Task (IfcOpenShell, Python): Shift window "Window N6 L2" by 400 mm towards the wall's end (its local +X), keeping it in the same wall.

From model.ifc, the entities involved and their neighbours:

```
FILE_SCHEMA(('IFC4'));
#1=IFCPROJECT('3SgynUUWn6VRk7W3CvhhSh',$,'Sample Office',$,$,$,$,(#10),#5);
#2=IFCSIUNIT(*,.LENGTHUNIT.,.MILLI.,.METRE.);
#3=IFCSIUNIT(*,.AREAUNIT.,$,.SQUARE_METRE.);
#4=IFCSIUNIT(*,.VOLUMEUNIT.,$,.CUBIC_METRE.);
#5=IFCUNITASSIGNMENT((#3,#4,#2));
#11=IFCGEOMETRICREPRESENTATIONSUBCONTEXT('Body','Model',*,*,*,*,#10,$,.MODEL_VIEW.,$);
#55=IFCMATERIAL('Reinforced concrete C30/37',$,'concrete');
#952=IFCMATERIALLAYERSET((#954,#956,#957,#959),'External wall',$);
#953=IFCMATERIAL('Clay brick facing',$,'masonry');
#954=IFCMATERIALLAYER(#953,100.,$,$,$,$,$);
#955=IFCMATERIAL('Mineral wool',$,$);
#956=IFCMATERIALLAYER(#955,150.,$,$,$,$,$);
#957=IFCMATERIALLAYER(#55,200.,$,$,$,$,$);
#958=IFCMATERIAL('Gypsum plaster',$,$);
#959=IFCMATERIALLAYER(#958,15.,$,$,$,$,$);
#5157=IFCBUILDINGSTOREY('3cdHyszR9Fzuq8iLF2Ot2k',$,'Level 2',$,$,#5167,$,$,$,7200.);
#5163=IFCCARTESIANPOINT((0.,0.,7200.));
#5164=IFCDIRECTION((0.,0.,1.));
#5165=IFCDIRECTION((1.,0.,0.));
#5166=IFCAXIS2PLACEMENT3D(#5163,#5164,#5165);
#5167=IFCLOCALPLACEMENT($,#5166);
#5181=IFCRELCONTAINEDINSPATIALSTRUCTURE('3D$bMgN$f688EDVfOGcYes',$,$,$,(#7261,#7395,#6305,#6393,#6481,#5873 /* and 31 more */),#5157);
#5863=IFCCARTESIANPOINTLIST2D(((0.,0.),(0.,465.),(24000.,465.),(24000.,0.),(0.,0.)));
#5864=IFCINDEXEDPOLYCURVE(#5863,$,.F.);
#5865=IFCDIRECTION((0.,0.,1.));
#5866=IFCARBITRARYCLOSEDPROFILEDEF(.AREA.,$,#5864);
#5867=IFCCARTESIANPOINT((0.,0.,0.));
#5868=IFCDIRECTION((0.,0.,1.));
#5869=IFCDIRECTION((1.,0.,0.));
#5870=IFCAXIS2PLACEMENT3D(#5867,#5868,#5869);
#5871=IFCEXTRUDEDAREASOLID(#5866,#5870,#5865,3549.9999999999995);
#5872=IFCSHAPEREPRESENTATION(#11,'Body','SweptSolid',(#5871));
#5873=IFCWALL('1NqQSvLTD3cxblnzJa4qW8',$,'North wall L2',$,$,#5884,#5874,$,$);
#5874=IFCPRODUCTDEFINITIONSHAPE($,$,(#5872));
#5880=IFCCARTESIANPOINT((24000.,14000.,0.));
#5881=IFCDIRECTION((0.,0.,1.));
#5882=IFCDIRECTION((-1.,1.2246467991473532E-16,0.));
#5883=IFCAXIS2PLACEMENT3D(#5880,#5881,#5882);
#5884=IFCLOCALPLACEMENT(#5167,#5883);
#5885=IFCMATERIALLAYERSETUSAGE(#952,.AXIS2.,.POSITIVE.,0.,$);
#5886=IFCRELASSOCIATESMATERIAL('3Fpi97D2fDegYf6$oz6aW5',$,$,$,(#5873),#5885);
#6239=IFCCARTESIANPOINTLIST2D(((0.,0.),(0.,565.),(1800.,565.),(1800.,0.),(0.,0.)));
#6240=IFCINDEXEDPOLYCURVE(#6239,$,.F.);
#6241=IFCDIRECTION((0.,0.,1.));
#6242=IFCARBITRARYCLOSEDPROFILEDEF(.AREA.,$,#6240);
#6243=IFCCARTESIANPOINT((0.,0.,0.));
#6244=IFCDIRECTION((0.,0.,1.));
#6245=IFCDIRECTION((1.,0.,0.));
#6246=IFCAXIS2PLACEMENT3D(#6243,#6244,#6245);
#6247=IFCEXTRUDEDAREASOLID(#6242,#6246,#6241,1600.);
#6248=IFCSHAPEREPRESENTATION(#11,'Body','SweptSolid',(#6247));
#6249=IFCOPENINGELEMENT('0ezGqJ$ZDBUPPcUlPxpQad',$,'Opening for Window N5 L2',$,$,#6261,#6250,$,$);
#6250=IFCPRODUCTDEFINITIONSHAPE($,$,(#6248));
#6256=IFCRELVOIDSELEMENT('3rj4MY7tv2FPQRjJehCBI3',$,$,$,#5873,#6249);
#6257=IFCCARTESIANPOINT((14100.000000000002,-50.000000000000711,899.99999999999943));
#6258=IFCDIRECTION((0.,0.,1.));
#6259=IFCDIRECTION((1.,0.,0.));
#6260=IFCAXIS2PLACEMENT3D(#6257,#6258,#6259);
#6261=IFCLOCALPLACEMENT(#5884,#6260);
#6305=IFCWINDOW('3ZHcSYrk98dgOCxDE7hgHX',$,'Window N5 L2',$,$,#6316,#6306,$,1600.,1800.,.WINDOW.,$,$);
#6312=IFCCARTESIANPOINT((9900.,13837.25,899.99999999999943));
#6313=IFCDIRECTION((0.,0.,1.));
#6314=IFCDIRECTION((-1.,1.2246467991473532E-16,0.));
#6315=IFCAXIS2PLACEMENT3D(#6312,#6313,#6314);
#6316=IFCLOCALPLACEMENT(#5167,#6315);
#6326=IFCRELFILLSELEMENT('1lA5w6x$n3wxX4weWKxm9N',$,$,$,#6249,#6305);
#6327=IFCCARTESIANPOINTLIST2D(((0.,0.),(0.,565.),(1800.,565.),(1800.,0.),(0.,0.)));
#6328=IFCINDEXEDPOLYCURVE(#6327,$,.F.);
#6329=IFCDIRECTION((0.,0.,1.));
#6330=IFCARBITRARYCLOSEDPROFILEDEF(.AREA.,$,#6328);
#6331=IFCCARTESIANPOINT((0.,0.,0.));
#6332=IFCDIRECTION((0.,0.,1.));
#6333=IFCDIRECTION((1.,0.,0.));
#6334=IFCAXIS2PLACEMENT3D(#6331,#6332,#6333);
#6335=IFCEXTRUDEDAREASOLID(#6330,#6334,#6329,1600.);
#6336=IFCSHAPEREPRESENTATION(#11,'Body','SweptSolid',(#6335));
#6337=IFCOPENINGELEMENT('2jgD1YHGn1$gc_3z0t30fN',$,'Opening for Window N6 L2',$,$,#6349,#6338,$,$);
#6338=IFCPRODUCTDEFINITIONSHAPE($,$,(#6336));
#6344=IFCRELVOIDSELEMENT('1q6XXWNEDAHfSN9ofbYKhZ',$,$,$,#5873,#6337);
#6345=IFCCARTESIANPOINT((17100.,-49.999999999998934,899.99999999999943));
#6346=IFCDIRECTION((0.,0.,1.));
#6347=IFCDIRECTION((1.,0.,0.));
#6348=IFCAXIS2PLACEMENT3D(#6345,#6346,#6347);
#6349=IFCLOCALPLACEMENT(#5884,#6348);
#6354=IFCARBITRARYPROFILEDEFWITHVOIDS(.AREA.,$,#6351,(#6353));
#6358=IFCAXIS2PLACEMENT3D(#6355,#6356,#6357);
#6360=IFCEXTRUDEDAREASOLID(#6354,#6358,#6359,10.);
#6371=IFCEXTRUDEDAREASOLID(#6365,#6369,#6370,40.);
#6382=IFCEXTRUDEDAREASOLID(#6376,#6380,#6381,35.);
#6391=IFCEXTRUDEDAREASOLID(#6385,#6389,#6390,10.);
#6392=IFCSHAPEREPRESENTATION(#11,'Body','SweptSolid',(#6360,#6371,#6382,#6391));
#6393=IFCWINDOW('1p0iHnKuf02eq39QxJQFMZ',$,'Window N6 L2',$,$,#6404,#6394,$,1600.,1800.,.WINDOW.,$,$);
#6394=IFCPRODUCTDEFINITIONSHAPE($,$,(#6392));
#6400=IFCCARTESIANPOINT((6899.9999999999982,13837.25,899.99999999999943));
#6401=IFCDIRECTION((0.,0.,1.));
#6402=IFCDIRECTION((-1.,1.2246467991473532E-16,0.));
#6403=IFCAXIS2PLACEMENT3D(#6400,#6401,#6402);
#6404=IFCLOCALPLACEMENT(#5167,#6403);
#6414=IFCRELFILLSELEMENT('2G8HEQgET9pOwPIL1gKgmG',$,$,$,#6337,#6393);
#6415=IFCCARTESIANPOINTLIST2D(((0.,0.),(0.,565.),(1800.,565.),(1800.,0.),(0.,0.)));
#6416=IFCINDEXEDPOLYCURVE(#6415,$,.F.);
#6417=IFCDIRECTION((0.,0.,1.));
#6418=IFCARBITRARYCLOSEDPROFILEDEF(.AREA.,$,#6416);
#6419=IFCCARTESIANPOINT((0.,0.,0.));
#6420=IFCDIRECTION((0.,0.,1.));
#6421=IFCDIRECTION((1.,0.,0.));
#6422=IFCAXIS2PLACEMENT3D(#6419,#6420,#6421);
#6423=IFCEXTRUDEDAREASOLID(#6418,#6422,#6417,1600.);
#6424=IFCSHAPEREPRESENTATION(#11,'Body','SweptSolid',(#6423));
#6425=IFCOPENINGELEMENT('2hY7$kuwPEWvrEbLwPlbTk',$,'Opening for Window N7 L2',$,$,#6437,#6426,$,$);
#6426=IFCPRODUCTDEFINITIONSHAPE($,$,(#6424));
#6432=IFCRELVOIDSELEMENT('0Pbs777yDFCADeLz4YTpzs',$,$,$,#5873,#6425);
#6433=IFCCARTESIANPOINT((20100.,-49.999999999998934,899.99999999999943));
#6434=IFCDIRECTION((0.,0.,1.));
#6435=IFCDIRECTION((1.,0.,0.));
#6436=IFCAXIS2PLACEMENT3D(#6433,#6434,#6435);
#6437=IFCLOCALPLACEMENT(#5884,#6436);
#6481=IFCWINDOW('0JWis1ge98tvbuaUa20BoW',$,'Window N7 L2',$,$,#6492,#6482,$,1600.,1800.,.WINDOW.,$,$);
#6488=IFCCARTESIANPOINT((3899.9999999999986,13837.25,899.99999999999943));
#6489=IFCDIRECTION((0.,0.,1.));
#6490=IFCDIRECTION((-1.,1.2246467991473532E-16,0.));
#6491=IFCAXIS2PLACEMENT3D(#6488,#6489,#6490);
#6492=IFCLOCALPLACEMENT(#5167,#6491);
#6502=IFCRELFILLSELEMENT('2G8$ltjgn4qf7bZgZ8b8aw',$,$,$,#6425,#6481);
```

```python
import ifcopenshell
import ifcopenshell.api.geometry
import ifcopenshell.util.placement
import ifcopenshell.util.unit

model = ifcopenshell.open("model.ifc")
unit_scale = ifcopenshell.util.unit.calculate_unit_scale(model)

window = model.by_guid("1p0iHnKuf02eq39QxJQFMZ")
opening = window.FillsVoids[0].RelatingOpeningElement
wall = opening.VoidsElements[0].RelatingBuildingElement

wall_matrix = ifcopenshell.util.placement.get_local_placement(wall.ObjectPlacement)
shift = wall_matrix[:3, 0] * 0.4 / unit_scale
before = ifcopenshell.util.placement.get_local_placement(window.ObjectPlacement)[:3, 3].copy()

# The window is not placed relative to its opening, so move both.
for product in (opening, window):
    matrix = ifcopenshell.util.placement.get_local_placement(product.ObjectPlacement)
    matrix[:3, 3] += shift
    ifcopenshell.api.geometry.edit_object_placement(model, product=product, matrix=matrix, is_si=False)

after = ifcopenshell.util.placement.get_local_placement(window.ObjectPlacement)[:3, 3]
print("window moved by", (after - before).round(3) + 0.0)

model.write("model_updated.ifc")
```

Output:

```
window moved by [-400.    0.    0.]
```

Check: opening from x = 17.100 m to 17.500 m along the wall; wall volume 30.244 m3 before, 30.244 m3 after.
